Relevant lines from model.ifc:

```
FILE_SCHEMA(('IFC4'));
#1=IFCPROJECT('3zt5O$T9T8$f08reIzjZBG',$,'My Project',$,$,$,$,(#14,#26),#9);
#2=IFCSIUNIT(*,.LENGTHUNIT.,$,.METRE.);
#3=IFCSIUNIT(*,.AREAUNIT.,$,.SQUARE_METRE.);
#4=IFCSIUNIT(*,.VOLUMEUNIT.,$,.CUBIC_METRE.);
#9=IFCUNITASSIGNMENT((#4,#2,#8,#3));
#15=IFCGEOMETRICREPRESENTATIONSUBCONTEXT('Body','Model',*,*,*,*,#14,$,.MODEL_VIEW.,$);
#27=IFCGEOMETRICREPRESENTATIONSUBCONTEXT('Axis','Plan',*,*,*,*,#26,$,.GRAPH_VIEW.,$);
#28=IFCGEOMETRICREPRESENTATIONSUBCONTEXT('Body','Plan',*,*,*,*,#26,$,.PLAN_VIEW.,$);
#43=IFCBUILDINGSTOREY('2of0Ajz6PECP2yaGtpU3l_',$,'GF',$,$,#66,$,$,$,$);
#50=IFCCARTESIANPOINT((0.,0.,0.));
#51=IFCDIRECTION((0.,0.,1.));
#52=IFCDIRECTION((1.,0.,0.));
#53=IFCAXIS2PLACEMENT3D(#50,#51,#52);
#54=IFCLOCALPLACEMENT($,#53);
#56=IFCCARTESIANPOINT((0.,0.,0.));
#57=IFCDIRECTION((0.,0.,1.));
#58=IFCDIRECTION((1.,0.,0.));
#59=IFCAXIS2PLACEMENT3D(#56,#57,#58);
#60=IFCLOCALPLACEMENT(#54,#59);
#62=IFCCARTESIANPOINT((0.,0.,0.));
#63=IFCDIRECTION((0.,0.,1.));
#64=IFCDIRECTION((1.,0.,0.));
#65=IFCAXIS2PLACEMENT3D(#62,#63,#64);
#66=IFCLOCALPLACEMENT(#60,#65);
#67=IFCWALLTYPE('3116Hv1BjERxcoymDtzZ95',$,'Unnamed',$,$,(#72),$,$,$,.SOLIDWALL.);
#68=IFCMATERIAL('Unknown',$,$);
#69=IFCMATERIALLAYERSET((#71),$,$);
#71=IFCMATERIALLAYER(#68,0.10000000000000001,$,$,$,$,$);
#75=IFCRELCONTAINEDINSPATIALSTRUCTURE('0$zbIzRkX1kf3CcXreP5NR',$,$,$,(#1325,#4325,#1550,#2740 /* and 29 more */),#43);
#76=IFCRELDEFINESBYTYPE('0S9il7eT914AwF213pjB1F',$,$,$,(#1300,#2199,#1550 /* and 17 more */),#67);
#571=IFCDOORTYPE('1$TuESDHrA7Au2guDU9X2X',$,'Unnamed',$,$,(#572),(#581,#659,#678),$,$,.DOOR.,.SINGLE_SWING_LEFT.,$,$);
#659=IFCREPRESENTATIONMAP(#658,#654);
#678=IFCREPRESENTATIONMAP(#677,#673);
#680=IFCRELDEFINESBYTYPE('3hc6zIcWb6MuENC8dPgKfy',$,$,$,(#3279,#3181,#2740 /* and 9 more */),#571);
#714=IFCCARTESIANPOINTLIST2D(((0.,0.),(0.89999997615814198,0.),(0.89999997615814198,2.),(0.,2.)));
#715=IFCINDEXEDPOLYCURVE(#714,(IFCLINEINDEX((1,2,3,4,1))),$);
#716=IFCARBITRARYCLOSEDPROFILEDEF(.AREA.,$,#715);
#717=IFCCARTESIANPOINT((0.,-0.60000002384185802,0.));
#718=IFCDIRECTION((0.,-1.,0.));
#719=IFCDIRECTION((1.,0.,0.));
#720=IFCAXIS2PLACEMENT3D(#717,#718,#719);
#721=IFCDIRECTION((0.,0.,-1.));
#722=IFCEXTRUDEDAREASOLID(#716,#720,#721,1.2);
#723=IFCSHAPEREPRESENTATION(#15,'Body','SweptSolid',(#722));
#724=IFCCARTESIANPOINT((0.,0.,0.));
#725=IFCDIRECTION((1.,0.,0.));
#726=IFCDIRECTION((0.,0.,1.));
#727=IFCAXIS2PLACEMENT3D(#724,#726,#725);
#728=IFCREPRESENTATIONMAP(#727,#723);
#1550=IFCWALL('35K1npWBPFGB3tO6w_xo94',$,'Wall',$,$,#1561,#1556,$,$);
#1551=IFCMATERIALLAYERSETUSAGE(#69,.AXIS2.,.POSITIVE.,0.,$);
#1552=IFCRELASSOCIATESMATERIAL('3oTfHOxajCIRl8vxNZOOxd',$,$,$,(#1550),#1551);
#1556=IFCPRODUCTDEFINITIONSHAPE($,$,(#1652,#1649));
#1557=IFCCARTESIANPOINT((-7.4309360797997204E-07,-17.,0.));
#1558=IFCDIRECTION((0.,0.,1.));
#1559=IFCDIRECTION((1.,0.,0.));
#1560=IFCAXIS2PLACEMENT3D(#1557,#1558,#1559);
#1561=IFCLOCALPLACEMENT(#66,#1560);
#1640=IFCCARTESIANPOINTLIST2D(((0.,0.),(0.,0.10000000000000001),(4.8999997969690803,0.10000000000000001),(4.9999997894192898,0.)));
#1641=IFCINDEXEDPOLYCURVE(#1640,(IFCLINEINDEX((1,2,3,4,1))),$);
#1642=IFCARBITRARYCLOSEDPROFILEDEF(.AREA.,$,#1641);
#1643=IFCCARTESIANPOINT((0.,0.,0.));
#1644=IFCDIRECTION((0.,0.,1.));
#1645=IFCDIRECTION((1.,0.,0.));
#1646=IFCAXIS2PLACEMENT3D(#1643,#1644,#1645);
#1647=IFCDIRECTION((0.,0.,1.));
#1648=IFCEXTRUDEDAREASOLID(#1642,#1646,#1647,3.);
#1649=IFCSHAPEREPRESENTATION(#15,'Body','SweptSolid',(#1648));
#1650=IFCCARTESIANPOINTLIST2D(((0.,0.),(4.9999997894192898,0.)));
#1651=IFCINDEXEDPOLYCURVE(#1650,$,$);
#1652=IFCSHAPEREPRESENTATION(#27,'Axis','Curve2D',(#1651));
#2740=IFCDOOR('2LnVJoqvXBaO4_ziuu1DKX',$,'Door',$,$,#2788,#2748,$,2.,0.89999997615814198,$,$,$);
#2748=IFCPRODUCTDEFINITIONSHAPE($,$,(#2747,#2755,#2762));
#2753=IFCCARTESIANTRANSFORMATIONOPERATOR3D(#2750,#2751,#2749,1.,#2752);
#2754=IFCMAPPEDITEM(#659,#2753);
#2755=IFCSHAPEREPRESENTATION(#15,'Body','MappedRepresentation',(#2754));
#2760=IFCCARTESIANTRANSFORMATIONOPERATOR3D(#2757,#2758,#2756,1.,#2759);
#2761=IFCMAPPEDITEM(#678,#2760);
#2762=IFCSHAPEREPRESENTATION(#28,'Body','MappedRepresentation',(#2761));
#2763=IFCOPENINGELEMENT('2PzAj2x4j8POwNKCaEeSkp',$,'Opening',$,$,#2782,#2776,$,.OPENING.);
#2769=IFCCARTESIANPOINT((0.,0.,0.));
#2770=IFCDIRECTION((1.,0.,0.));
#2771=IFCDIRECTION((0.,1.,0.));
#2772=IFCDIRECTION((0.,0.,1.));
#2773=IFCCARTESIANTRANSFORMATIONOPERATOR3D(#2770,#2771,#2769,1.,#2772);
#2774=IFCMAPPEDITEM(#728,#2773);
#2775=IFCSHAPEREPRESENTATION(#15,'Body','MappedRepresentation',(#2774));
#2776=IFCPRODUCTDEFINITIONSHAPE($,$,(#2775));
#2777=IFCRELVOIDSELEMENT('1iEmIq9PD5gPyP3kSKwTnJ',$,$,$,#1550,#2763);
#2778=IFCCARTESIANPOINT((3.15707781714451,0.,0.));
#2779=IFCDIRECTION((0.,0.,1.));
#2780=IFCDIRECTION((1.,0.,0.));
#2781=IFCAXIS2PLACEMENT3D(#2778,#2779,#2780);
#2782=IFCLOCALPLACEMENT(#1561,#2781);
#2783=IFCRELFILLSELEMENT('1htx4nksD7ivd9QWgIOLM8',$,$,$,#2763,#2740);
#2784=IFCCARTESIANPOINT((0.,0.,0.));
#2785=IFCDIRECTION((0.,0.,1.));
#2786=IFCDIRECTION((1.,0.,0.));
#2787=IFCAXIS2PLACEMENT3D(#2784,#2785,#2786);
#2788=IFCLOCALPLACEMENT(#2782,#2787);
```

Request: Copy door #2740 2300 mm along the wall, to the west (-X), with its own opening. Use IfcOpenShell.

```python
import ifcopenshell
import ifcopenshell.api.feature
import ifcopenshell.api.geometry
import ifcopenshell.api.root
import ifcopenshell.geom
import ifcopenshell.util.element
import ifcopenshell.util.placement
import ifcopenshell.util.shape
import ifcopenshell.util.unit

model = ifcopenshell.open("model.ifc")
unit_scale = ifcopenshell.util.unit.calculate_unit_scale(model)
settings = ifcopenshell.geom.settings()


def volume(element):
    """Net volume in cubic metres, openings subtracted."""
    shape = ifcopenshell.geom.create_shape(settings, element)
    return ifcopenshell.util.shape.get_volume(shape.geometry)


door = model.by_guid("2LnVJoqvXBaO4_ziuu1DKX")
opening = door.FillsVoids[0].RelatingOpeningElement
wall = opening.VoidsElements[0].RelatingBuildingElement
before = volume(wall)
shift = ifcopenshell.util.placement.get_local_placement(wall.ObjectPlacement)[:3, 0] * -2.3 / unit_scale

# copy_class copies the void relationship, type, container and properties, but no geometry.
new_opening = ifcopenshell.api.root.copy_class(model, product=opening)
new_opening.Representation = ifcopenshell.util.element.copy_deep(
    model, opening.Representation, exclude=["IfcGeometricRepresentationContext", "IfcRepresentationMap"]
)
new_door = ifcopenshell.api.root.copy_class(model, product=door)
new_door.Representation = ifcopenshell.util.element.copy_deep(
    model, door.Representation, exclude=["IfcGeometricRepresentationContext", "IfcRepresentationMap"]
)
ifcopenshell.api.feature.add_filling(model, opening=new_opening, element=new_door)

for old, new in ((opening, new_opening), (door, new_door)):
    matrix = ifcopenshell.util.placement.get_local_placement(old.ObjectPlacement)
    matrix[:3, 3] += shift
    ifcopenshell.api.geometry.edit_object_placement(model, product=new, matrix=matrix, is_si=False)

after = volume(wall)

print(f"wall volume {before:.3f} -> {after:.3f} m3")

model.write("model_v2.ifc")
```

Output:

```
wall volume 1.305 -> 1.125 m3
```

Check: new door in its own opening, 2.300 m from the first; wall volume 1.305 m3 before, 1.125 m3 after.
